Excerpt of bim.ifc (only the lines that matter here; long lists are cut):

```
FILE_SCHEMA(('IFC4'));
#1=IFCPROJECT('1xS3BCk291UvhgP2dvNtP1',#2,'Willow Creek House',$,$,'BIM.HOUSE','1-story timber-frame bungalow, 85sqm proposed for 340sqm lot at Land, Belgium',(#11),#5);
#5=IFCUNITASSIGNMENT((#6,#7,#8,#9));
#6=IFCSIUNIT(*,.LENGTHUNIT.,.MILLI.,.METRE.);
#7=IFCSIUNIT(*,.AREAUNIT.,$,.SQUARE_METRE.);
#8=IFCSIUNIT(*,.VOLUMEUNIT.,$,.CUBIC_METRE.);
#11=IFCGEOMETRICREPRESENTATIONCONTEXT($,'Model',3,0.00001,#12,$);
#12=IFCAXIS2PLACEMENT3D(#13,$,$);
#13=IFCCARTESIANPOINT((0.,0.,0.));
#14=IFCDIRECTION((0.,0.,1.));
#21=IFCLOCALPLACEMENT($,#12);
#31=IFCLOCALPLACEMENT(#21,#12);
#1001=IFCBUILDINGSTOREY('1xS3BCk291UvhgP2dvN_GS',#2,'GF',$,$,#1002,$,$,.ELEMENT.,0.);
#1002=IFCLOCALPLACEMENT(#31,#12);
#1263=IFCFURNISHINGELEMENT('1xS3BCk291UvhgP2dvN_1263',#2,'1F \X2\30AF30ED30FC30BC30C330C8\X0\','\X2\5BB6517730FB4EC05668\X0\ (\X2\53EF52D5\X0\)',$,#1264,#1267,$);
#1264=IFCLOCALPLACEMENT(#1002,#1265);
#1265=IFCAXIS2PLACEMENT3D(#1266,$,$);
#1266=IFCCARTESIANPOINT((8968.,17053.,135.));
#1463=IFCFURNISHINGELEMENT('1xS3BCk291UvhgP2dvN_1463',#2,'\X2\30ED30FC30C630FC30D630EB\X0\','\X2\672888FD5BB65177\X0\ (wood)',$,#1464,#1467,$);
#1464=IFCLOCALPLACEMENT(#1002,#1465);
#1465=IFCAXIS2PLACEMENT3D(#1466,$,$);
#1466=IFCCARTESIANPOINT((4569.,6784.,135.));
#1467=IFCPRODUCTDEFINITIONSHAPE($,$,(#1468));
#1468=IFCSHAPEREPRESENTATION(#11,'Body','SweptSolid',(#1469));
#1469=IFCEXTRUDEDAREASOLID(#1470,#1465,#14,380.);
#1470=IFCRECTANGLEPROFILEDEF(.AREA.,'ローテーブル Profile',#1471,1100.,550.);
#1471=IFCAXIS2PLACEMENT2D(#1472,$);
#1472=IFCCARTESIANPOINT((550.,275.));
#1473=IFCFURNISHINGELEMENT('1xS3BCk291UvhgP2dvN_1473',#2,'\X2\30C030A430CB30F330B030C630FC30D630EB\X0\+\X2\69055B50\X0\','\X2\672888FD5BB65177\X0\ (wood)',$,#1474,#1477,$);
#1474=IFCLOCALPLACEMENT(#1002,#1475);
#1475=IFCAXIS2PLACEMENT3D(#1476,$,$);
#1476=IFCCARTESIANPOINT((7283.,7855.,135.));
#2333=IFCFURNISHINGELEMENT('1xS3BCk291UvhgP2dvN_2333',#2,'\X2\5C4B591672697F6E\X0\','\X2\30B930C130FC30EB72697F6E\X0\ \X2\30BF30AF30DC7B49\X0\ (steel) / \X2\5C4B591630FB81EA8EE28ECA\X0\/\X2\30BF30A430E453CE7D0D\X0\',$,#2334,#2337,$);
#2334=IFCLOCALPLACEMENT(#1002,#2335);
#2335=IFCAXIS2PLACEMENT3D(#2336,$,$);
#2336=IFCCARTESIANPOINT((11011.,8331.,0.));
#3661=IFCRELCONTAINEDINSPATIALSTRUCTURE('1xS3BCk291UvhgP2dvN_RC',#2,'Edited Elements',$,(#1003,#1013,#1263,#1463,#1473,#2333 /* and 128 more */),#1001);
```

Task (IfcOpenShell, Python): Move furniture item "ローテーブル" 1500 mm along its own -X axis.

```python
import ifcopenshell
import ifcopenshell.api.geometry
import ifcopenshell.util.placement

model = ifcopenshell.open("bim.ifc")

item = model.by_guid("1xS3BCk291UvhgP2dvN_1463")
matrix = ifcopenshell.util.placement.get_local_placement(item.ObjectPlacement)
matrix[:3, 3] -= matrix[:3, 0] * 1500.0
ifcopenshell.api.geometry.edit_object_placement(model, product=item, matrix=matrix, is_si=False)

print(ifcopenshell.util.placement.get_local_placement(item.ObjectPlacement).round(3) + 0.0)

model.write("bim_v2.ifc")
```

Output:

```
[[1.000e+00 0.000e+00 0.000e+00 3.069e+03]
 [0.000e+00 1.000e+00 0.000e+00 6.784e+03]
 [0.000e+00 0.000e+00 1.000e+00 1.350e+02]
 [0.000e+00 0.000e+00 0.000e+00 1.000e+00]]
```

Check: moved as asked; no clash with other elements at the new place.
